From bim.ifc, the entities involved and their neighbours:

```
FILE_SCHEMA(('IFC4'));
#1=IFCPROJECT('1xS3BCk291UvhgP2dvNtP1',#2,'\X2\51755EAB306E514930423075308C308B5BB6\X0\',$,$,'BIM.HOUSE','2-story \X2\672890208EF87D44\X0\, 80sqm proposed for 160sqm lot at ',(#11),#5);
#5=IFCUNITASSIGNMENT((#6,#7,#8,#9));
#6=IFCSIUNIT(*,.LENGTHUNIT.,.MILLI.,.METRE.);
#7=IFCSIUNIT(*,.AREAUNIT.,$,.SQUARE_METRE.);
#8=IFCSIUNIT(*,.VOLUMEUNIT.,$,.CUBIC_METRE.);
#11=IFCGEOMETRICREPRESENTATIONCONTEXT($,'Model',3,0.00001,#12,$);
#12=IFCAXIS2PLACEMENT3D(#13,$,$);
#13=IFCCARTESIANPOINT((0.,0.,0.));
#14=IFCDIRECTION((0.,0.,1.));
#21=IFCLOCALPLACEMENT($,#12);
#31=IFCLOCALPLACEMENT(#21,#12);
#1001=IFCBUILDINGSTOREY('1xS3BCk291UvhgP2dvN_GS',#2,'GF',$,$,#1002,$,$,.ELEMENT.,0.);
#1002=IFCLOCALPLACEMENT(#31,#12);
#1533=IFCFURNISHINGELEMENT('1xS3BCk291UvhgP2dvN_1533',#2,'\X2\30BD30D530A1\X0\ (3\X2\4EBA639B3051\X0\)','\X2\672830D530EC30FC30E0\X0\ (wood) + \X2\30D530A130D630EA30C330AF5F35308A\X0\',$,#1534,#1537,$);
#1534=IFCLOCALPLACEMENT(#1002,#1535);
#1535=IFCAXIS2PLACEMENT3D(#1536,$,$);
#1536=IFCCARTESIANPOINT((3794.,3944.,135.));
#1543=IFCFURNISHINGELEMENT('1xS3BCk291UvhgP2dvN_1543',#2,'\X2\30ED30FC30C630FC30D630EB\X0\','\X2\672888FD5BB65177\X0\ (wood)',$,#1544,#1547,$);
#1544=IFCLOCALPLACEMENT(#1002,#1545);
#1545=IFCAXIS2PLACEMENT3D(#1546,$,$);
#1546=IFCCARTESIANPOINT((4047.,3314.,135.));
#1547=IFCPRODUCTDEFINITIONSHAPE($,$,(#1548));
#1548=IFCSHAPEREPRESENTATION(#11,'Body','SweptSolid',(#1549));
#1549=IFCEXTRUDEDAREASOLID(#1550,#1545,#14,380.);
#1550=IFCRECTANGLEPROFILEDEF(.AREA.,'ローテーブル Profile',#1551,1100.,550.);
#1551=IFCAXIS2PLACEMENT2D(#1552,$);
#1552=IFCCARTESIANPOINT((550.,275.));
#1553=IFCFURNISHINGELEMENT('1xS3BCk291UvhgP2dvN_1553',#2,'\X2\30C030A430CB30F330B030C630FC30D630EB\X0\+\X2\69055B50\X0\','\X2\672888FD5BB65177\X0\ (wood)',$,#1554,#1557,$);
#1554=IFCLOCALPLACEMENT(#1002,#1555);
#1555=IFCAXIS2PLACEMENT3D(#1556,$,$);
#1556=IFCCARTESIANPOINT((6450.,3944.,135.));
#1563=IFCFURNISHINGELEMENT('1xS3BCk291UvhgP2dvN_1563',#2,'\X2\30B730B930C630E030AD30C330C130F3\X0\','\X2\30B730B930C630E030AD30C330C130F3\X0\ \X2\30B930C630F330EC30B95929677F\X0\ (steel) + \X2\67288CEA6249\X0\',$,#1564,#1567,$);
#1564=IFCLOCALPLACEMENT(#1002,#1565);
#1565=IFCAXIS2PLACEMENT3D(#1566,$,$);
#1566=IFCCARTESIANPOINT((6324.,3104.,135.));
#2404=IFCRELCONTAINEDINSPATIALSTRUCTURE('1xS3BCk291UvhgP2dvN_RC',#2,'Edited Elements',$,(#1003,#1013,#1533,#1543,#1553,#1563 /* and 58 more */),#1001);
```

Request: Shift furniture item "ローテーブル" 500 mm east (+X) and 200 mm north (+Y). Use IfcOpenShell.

```python
import ifcopenshell
import ifcopenshell.api.geometry
import ifcopenshell.util.placement

model = ifcopenshell.open("bim.ifc")

item = model.by_guid("1xS3BCk291UvhgP2dvN_1543")
matrix = ifcopenshell.util.placement.get_local_placement(item.ObjectPlacement)
matrix[0, 3] += 500.0
matrix[1, 3] += 200.0
ifcopenshell.api.geometry.edit_object_placement(model, product=item, matrix=matrix, is_si=False)

print(ifcopenshell.util.placement.get_local_placement(item.ObjectPlacement).round(3) + 0.0)

model.write("bim_rev.ifc")
```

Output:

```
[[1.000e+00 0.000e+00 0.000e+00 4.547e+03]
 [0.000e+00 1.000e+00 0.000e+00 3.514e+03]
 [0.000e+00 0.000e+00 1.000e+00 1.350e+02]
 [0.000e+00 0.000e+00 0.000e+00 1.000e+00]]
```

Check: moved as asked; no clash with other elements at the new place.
